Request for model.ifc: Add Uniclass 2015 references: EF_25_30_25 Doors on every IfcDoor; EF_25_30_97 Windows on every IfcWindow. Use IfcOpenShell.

First a look at what the model holds.

```python
import ifcopenshell

model = ifcopenshell.open("model.ifc")
print(model.schema)
print("classifications:", [c.Name for c in model.by_type("IfcClassification")])
for ifc_class in ("IfcDoor", "IfcRoof", "IfcStair", "IfcWall", "IfcWindow"):
    print(ifc_class, len(model.by_type(ifc_class)))
```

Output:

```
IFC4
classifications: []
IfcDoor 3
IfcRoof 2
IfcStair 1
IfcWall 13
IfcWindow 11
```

```python
import ifcopenshell
import ifcopenshell.api.classification

model = ifcopenshell.open("model.ifc")

system = ifcopenshell.api.classification.add_classification(model, classification="Uniclass 2015")

codes = {
    "IfcDoor": ("EF_25_30_25", "Doors"),
    "IfcWindow": ("EF_25_30_97", "Windows"),
}
for ifc_class, (code, name) in codes.items():
    products = model.by_type(ifc_class)
    ifcopenshell.api.classification.add_reference(
        model, products=products, classification=system, identification=code, name=name
    )
    print(code, len(products))

model.write("model_v2.ifc")
```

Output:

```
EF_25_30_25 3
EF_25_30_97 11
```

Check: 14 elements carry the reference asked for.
